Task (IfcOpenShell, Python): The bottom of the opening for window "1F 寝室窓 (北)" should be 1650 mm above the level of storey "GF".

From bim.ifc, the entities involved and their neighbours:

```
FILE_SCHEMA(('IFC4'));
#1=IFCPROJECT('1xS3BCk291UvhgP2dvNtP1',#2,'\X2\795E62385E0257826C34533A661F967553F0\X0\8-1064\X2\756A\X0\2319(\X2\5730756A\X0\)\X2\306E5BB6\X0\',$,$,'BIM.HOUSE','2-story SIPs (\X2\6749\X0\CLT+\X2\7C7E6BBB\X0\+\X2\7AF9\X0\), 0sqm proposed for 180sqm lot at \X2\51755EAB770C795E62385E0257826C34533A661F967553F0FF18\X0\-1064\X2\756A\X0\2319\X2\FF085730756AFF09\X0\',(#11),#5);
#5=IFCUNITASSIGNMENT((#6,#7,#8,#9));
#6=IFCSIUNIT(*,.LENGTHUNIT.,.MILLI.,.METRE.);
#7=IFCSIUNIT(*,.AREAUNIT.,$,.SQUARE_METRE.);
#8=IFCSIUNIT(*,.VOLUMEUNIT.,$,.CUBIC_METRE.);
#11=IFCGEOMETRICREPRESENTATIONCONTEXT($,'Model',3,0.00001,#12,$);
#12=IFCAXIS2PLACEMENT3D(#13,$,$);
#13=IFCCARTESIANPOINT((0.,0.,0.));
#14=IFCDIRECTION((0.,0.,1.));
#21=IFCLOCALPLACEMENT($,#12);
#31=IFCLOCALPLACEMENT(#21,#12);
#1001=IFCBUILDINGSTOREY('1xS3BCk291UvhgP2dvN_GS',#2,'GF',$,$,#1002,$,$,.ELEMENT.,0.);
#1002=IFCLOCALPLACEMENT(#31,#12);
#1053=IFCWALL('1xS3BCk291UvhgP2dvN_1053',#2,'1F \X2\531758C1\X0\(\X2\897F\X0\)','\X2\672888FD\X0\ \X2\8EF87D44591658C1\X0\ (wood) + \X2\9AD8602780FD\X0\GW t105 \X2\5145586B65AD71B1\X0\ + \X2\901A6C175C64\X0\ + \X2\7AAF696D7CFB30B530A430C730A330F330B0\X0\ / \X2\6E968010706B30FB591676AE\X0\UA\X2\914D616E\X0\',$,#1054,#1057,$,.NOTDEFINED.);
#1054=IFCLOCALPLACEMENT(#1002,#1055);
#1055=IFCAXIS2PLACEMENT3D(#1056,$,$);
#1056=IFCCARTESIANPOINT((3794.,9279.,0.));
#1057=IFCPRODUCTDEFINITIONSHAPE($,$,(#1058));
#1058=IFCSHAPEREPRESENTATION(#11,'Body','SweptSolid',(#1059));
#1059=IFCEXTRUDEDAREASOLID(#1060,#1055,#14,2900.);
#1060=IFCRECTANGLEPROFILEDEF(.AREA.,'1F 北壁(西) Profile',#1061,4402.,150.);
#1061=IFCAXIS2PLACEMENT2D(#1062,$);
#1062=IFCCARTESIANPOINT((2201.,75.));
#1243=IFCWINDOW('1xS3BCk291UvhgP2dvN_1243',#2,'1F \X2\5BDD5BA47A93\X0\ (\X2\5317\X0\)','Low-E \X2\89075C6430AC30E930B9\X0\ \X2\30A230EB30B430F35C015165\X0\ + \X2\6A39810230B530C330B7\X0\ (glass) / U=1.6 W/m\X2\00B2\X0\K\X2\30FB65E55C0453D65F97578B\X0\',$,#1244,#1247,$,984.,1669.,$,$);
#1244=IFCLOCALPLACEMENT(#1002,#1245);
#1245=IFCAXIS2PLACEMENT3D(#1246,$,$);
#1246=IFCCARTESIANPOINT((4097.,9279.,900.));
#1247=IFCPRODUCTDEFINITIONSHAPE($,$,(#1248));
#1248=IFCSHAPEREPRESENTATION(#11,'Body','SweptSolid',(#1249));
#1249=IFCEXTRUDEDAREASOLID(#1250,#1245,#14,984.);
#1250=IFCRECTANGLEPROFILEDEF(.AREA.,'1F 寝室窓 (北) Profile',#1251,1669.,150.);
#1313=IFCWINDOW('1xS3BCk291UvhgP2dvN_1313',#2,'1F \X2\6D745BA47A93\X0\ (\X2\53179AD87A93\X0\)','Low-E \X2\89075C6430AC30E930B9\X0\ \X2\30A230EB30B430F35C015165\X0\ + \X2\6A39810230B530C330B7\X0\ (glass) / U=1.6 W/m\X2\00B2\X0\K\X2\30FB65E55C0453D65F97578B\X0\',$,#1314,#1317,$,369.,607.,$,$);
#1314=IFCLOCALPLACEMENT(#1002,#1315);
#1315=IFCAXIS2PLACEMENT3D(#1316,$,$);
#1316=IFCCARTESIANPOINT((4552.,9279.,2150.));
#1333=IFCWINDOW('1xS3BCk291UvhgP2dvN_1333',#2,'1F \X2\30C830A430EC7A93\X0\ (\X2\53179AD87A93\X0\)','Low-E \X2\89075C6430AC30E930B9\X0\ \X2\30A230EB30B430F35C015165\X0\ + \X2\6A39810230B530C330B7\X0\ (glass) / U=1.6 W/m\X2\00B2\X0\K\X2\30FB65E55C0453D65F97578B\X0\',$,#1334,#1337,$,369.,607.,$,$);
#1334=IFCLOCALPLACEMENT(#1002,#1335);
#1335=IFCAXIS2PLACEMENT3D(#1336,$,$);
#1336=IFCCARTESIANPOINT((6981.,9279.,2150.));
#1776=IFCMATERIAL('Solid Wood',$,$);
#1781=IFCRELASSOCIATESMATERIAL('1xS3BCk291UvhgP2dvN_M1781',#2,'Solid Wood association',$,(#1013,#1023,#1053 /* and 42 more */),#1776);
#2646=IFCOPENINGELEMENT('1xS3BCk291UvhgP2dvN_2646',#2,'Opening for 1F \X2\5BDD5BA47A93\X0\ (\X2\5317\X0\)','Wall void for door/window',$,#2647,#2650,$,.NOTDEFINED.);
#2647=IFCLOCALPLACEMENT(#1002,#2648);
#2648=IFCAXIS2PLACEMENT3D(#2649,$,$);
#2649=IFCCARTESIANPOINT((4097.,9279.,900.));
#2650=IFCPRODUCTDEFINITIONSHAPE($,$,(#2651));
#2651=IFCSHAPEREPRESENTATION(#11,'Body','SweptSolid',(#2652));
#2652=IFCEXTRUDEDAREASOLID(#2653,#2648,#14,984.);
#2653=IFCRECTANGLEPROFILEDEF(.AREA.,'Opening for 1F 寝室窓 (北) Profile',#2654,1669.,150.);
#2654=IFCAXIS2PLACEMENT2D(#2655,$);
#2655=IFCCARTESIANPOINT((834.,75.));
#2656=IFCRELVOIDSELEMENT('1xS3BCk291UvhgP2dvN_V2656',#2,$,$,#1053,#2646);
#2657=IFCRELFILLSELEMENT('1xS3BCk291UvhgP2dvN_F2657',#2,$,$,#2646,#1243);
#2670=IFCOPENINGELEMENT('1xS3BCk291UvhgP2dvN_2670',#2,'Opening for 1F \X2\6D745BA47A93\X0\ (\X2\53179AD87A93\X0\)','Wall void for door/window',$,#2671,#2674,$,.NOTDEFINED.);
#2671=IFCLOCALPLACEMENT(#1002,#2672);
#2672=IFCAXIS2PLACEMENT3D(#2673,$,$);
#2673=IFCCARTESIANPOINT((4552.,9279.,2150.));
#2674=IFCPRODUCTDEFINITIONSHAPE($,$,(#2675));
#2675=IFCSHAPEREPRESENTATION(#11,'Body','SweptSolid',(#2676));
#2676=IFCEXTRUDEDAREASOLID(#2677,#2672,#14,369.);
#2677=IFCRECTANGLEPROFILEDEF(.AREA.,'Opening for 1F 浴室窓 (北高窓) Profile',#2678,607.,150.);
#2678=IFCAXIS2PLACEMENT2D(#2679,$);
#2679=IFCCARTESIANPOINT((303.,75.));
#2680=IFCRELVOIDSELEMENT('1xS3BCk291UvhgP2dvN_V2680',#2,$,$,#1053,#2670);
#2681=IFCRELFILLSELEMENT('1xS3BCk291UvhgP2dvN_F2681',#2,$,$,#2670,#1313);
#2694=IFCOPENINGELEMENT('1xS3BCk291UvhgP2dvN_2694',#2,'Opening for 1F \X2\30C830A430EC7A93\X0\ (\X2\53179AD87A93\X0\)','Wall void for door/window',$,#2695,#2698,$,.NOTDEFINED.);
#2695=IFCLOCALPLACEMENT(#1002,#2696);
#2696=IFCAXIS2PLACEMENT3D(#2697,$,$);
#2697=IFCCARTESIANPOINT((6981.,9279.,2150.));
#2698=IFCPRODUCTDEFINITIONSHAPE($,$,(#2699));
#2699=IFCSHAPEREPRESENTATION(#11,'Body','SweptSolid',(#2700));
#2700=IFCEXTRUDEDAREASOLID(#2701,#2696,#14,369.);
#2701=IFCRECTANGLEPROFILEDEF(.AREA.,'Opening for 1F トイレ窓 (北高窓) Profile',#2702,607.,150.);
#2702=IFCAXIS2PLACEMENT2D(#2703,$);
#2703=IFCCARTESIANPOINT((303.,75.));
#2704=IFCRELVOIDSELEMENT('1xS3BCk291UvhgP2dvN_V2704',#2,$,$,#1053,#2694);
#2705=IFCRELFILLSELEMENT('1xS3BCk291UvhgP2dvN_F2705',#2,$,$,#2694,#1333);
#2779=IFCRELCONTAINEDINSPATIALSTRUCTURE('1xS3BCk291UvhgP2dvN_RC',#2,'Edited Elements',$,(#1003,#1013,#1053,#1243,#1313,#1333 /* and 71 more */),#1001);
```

```python
import numpy as np
import ifcopenshell
import ifcopenshell.api.geometry
import ifcopenshell.geom
import ifcopenshell.util.element
import ifcopenshell.util.placement
import ifcopenshell.util.shape
import ifcopenshell.util.unit

model = ifcopenshell.open("bim.ifc")
unit_scale = ifcopenshell.util.unit.calculate_unit_scale(model)

window = model.by_guid("1xS3BCk291UvhgP2dvN_1243")
opening = window.FillsVoids[0].RelatingOpeningElement
storey = ifcopenshell.util.element.get_container(window, ifc_class="IfcBuildingStorey")
level = ifcopenshell.util.placement.get_local_placement(storey.ObjectPlacement)[2, 3]

# The opening's origin need not be at the sill, so measure its lowest point.
shape = ifcopenshell.geom.create_shape(ifcopenshell.geom.settings(), opening)
bottom = ifcopenshell.util.shape.get_shape_bottom_elevation(shape, shape.geometry) / unit_scale
dz = level + 1.65 / unit_scale - bottom

shift = np.array([0.0, 0.0, dz])
# The window is not placed relative to its opening, so move both.
for product in (opening, window):
    matrix = ifcopenshell.util.placement.get_local_placement(product.ObjectPlacement)
    matrix[:3, 3] += shift
    ifcopenshell.api.geometry.edit_object_placement(model, product=product, matrix=matrix, is_si=False)

print(f"moved by {dz * unit_scale:+.3f} m")

model.write("bim_v2.ifc")
```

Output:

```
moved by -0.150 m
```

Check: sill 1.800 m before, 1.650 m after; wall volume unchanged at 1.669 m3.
